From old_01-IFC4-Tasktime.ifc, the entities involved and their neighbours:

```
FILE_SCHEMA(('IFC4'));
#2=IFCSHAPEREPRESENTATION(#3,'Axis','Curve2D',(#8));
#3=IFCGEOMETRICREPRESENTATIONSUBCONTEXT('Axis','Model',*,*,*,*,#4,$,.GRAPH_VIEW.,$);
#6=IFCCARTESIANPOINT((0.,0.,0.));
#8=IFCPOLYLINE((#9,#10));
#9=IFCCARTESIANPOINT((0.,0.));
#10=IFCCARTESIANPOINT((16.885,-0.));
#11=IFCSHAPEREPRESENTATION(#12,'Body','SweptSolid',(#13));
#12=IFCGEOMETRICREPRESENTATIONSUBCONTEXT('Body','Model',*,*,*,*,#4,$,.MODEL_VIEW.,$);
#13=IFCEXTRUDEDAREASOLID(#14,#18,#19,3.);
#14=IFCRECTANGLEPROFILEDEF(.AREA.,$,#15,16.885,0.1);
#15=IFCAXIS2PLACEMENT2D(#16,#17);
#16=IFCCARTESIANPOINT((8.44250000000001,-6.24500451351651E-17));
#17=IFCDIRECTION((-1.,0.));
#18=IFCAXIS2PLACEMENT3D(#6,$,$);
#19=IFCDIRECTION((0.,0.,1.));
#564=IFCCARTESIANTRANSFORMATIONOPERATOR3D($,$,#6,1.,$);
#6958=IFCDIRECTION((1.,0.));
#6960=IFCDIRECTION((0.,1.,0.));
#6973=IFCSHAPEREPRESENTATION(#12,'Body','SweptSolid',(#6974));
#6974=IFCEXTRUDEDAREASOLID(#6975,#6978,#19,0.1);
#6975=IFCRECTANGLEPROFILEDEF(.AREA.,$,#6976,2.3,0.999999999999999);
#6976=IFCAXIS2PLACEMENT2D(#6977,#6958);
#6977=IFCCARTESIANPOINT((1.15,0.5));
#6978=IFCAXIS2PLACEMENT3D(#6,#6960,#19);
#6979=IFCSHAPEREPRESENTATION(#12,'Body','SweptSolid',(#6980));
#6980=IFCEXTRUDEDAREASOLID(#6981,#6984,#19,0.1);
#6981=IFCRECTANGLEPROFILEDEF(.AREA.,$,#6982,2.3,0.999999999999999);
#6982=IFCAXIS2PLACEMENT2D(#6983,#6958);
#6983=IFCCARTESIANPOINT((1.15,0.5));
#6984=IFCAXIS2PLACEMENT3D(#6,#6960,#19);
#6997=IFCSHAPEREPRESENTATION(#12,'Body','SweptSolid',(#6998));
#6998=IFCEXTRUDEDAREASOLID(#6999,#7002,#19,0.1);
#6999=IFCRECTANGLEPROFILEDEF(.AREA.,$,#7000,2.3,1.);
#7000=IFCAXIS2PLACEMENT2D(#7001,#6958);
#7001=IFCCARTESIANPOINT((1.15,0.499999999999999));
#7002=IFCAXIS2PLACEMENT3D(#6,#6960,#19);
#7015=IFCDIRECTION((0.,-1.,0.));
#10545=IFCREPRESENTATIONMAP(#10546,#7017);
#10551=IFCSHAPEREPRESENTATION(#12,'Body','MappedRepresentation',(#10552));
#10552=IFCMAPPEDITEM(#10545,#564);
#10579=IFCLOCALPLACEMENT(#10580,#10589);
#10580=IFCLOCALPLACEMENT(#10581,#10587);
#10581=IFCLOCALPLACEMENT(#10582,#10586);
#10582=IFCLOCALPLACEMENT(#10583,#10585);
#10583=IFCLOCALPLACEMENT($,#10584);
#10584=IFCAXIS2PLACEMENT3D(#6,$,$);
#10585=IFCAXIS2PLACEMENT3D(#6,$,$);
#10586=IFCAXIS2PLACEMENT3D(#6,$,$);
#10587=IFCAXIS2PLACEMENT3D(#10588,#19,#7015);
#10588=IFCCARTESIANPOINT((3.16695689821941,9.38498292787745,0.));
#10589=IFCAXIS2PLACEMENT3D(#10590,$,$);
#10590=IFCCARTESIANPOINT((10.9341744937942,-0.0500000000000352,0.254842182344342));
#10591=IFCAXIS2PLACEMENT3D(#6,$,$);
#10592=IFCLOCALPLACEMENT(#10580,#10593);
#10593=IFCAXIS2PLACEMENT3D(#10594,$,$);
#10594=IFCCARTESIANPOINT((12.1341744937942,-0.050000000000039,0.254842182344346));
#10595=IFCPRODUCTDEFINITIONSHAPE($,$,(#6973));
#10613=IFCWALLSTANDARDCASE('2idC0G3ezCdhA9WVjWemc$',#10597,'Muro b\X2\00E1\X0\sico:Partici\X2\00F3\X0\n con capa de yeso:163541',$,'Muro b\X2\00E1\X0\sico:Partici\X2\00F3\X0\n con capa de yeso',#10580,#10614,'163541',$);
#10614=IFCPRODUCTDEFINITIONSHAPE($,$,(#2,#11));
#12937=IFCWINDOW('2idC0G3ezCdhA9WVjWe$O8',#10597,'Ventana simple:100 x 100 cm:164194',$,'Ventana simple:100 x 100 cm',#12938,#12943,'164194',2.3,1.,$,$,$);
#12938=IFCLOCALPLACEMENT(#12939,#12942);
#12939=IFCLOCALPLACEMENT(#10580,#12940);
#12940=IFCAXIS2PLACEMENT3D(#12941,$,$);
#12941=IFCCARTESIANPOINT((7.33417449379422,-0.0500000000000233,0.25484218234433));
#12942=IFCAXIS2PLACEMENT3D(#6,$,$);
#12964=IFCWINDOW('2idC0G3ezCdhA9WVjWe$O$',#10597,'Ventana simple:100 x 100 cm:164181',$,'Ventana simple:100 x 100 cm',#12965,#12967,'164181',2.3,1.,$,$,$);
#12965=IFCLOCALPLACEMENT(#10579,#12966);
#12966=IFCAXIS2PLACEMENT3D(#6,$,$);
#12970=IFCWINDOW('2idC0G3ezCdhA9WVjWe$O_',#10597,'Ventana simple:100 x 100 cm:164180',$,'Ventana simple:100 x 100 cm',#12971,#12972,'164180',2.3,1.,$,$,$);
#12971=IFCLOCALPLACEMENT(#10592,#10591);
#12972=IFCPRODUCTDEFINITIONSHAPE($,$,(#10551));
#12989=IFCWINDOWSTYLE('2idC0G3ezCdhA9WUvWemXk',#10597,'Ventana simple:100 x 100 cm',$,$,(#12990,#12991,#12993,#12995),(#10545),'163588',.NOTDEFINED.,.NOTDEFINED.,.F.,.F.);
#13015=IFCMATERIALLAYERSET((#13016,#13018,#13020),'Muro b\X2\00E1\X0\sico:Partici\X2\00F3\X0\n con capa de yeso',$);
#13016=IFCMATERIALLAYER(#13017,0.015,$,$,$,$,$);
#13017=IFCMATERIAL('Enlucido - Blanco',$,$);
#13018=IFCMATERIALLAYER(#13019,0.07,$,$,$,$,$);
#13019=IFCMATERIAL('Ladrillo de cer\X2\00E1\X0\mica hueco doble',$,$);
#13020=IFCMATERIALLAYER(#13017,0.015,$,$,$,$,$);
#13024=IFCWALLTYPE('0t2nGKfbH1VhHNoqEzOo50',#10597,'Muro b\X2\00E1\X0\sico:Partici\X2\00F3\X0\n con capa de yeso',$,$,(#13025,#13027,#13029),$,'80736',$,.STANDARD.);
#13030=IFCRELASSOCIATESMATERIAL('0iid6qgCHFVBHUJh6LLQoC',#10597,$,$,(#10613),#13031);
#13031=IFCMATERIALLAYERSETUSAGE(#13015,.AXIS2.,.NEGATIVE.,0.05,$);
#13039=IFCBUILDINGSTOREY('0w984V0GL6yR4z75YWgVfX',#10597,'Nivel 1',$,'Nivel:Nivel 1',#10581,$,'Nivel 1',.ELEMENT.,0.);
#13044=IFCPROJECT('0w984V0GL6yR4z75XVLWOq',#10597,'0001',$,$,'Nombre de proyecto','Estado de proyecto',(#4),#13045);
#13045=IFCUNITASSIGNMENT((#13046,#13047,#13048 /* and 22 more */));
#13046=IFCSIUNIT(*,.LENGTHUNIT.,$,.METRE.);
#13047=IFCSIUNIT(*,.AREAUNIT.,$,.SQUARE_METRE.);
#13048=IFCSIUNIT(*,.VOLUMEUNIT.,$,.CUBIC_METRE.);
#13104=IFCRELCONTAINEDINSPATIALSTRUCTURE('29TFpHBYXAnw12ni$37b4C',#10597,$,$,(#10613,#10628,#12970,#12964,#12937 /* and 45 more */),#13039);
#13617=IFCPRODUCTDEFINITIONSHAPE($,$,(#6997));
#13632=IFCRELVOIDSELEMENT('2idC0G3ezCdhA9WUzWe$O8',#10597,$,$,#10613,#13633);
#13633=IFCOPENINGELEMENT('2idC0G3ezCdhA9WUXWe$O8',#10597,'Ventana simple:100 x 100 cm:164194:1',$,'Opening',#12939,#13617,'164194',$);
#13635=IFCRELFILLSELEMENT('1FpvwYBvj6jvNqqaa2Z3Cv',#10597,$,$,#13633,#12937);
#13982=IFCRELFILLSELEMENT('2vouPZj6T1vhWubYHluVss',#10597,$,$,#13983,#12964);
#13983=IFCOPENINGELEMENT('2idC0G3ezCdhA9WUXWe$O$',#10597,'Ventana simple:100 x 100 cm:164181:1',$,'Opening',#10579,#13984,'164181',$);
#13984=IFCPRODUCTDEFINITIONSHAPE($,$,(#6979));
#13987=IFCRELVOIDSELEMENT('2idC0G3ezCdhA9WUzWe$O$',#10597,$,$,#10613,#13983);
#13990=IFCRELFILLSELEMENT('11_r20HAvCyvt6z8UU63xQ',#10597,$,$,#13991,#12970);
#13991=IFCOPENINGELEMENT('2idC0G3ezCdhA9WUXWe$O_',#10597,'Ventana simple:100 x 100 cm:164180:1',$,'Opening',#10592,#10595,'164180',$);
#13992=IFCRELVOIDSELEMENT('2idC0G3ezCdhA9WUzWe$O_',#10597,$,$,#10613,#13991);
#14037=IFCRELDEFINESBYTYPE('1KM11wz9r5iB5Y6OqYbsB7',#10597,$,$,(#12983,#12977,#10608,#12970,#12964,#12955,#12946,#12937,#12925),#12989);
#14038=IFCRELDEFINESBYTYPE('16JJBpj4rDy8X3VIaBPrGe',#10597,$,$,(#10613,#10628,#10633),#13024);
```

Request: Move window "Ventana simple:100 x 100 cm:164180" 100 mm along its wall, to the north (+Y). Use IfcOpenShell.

```python
import ifcopenshell
import ifcopenshell.api.geometry
import ifcopenshell.util.placement
import ifcopenshell.util.unit

model = ifcopenshell.open("old_01-IFC4-Tasktime.ifc")
unit_scale = ifcopenshell.util.unit.calculate_unit_scale(model)

window = model.by_guid("2idC0G3ezCdhA9WVjWe$O_")
opening = window.FillsVoids[0].RelatingOpeningElement
wall = opening.VoidsElements[0].RelatingBuildingElement

wall_matrix = ifcopenshell.util.placement.get_local_placement(wall.ObjectPlacement)
shift = wall_matrix[:3, 0] * -0.1 / unit_scale
before = ifcopenshell.util.placement.get_local_placement(window.ObjectPlacement)[:3, 3].copy()

# The window is placed relative to its opening, so it follows when the opening moves.
matrix = ifcopenshell.util.placement.get_local_placement(opening.ObjectPlacement)
matrix[:3, 3] += shift
ifcopenshell.api.geometry.edit_object_placement(
    model, product=opening, matrix=matrix, is_si=False, should_transform_children=True
)

after = ifcopenshell.util.placement.get_local_placement(window.ObjectPlacement)[:3, 3]
print("window moved by", (after - before).round(3) + 0.0)

model.write("old_01-IFC4-Tasktime_edited.ifc")
```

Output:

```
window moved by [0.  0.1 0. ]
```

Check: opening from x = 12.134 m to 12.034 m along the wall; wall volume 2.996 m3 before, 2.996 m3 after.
